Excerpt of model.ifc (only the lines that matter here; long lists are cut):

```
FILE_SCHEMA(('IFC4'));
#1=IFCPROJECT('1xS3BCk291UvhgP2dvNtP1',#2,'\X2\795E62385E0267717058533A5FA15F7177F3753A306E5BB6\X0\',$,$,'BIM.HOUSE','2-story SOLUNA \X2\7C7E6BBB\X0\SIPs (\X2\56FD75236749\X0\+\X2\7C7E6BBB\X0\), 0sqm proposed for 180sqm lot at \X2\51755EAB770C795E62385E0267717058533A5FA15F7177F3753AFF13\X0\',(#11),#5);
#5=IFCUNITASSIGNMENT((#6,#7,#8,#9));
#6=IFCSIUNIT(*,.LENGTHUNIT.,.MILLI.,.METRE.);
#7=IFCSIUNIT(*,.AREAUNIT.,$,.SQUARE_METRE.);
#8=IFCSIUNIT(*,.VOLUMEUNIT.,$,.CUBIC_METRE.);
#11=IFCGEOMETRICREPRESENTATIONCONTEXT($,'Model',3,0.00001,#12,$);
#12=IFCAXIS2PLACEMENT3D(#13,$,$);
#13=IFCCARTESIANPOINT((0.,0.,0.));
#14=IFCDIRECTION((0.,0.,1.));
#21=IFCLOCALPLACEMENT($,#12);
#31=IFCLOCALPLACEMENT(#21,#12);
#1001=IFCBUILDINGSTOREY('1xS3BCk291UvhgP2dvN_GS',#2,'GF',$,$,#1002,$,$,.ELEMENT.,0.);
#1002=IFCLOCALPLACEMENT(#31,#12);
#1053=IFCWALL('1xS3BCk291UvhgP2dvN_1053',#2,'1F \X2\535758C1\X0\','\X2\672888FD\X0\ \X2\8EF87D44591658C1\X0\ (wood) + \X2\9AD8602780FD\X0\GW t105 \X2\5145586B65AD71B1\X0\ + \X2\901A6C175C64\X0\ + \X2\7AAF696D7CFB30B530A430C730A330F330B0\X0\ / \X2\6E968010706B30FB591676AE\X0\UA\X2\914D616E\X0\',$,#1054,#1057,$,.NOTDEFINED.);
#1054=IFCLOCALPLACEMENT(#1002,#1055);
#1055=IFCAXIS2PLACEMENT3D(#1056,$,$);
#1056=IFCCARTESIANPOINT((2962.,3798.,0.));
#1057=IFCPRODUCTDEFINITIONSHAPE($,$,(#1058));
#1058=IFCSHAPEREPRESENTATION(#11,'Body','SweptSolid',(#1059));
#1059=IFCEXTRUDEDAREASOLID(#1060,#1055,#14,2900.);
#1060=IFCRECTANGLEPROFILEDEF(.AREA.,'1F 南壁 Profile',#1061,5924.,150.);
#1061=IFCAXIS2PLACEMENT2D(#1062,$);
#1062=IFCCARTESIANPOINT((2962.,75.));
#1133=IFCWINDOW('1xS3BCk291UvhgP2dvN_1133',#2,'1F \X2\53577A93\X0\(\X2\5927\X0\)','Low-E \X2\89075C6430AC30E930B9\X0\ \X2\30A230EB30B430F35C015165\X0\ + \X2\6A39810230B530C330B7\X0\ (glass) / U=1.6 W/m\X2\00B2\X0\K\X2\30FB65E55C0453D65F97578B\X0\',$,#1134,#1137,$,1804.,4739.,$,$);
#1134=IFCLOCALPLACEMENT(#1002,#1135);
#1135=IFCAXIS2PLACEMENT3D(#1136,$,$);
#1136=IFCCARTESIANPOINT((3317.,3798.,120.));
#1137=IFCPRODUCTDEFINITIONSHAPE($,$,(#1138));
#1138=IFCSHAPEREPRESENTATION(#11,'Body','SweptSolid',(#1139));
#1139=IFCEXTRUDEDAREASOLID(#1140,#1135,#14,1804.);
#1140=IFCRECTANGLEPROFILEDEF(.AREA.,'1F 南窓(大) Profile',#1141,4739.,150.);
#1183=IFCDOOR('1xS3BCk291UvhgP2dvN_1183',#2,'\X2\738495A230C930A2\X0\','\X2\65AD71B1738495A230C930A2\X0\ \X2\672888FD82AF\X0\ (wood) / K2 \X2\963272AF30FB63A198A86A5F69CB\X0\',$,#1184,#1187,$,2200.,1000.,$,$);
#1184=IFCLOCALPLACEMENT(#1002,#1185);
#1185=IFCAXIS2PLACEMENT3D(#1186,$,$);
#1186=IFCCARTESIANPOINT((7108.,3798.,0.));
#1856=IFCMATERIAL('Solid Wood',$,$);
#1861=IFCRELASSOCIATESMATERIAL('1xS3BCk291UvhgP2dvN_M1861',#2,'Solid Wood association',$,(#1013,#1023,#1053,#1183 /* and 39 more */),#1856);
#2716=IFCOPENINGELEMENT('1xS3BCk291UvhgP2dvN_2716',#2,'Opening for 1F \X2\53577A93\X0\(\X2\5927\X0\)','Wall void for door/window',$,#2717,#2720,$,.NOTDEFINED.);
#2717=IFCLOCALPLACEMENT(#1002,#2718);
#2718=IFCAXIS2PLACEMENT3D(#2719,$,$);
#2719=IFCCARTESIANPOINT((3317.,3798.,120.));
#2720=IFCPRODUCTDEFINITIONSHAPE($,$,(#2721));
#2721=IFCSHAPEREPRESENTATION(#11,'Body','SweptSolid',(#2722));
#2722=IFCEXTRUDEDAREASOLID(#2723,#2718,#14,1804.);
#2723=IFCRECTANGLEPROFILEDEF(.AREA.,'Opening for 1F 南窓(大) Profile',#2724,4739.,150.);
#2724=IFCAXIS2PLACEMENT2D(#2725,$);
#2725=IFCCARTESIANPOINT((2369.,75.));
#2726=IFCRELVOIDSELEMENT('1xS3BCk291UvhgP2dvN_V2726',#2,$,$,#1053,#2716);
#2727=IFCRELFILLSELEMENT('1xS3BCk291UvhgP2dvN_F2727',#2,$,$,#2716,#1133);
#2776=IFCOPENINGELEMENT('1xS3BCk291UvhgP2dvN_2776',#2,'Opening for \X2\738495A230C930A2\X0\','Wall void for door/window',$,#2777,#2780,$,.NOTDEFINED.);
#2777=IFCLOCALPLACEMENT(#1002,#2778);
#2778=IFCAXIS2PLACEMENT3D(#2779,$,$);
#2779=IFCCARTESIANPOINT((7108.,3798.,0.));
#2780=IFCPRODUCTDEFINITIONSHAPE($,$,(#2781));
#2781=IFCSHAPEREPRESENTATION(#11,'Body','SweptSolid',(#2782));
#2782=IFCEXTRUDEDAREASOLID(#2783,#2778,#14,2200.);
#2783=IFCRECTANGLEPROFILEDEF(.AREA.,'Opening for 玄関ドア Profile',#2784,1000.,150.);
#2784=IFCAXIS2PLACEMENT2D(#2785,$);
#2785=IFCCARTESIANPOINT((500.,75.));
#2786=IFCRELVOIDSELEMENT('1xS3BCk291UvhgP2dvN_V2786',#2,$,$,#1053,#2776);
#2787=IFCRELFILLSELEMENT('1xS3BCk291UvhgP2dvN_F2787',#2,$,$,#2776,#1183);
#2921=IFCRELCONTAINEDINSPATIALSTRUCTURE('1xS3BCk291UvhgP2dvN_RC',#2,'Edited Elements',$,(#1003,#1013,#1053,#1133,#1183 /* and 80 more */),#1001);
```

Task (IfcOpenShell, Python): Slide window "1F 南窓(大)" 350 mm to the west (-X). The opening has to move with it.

```python
import ifcopenshell
import ifcopenshell.api.geometry
import ifcopenshell.util.placement
import ifcopenshell.util.unit

model = ifcopenshell.open("model.ifc")
unit_scale = ifcopenshell.util.unit.calculate_unit_scale(model)

window = model.by_id(1133)
opening = window.FillsVoids[0].RelatingOpeningElement
wall = opening.VoidsElements[0].RelatingBuildingElement

wall_matrix = ifcopenshell.util.placement.get_local_placement(wall.ObjectPlacement)
shift = wall_matrix[:3, 0] * -0.35 / unit_scale
before = ifcopenshell.util.placement.get_local_placement(window.ObjectPlacement)[:3, 3].copy()

# The window is not placed relative to its opening, so move both.
for product in (opening, window):
    matrix = ifcopenshell.util.placement.get_local_placement(product.ObjectPlacement)
    matrix[:3, 3] += shift
    ifcopenshell.api.geometry.edit_object_placement(model, product=product, matrix=matrix, is_si=False)

after = ifcopenshell.util.placement.get_local_placement(window.ObjectPlacement)[:3, 3]
print("window moved by", (after - before).round(3) + 0.0)

model.write("model_rev.ifc")
```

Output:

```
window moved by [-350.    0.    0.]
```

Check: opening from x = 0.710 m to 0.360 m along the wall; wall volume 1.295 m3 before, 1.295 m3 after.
